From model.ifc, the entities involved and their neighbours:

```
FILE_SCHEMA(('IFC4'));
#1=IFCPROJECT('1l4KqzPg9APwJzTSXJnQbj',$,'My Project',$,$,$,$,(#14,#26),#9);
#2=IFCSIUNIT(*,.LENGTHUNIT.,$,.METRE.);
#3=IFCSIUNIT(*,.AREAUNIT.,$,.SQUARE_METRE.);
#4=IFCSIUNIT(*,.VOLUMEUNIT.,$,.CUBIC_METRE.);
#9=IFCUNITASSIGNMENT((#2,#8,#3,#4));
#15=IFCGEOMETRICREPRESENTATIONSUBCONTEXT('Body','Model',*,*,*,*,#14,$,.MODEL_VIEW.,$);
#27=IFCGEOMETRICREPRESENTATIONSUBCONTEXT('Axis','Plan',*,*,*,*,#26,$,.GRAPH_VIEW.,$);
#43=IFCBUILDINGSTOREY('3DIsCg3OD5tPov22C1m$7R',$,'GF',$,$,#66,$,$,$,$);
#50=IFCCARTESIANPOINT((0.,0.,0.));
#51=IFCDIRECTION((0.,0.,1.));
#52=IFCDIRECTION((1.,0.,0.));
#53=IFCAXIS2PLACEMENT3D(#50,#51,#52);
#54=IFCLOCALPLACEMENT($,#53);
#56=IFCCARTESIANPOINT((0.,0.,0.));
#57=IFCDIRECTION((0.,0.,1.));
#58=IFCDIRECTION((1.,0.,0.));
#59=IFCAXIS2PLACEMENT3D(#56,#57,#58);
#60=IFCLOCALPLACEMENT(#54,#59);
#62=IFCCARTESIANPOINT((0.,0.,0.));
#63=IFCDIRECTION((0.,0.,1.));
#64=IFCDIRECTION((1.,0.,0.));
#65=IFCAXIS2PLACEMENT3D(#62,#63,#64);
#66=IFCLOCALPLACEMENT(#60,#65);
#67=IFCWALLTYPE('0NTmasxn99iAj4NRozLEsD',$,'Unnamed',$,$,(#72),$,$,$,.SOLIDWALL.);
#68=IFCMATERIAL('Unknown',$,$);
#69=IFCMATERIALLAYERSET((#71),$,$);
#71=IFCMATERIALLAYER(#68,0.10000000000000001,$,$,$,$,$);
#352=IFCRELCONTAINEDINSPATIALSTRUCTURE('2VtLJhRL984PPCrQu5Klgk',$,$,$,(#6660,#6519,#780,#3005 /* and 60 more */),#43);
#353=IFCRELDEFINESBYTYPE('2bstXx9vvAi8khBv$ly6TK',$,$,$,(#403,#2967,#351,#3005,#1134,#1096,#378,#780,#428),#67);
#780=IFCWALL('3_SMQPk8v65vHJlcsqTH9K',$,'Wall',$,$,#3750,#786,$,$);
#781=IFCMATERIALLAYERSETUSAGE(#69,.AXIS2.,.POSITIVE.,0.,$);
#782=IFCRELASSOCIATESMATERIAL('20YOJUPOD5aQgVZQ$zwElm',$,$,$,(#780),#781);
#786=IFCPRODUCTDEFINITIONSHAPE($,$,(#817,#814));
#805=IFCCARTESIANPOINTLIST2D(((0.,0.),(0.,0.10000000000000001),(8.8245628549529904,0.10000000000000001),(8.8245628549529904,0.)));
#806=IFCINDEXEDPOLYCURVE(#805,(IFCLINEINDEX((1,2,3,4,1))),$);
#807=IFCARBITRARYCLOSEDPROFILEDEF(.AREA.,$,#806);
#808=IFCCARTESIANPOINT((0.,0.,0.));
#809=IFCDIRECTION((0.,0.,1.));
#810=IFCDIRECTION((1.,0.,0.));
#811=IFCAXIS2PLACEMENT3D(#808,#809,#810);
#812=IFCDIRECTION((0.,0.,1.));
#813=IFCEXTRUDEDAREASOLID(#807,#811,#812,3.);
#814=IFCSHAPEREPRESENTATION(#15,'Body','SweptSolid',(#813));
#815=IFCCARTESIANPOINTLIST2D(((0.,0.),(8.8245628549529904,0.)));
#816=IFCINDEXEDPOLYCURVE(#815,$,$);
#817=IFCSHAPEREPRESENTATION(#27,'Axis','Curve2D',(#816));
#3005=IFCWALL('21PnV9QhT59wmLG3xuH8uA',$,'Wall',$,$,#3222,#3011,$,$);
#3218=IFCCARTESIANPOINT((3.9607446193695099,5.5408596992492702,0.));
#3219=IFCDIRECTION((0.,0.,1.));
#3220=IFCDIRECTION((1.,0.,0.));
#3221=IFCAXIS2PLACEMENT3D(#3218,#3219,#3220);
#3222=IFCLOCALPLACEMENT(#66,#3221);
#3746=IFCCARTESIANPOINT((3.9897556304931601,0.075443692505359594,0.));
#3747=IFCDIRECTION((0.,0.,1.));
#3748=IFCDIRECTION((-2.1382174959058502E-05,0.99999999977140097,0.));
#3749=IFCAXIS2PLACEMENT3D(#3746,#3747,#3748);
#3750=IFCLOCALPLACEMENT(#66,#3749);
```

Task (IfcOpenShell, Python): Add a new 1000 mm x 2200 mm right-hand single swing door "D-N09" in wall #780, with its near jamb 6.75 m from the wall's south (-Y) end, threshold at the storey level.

```python
import numpy as np
import ifcopenshell
import ifcopenshell.api.feature
import ifcopenshell.api.geometry
import ifcopenshell.api.root
import ifcopenshell.api.spatial
import ifcopenshell.geom
import ifcopenshell.util.element
import ifcopenshell.util.placement
import ifcopenshell.util.representation
import ifcopenshell.util.shape
import ifcopenshell.util.unit

model = ifcopenshell.open("model.ifc")
unit_scale = ifcopenshell.util.unit.calculate_unit_scale(model)
settings = ifcopenshell.geom.settings()


def volume(element):
    """Net volume in cubic metres, openings subtracted."""
    shape = ifcopenshell.geom.create_shape(settings, element)
    return ifcopenshell.util.shape.get_volume(shape.geometry)


wall = model.by_id(780)
storey = ifcopenshell.util.element.get_container(wall, ifc_class="IfcBuildingStorey")
context = ifcopenshell.util.representation.get_context(model, "Model", "Body", "MODEL_VIEW")
before = volume(wall)

width, height, from_end, sill = 1, 2.2, 6.75, 0.0  # metres

# The wall runs along its own X axis, and the end named is its -X end.
wall_shape = ifcopenshell.geom.create_shape(settings, wall)
x, y, z = ifcopenshell.util.shape.get_vertices(wall_shape.geometry).T
start = x.min() + from_end
face, thickness = float(y.min()), float(y.max() - y.min())
wall_matrix = ifcopenshell.util.placement.get_local_placement(wall.ObjectPlacement)
level = ifcopenshell.util.placement.get_local_placement(storey.ObjectPlacement)[2, 3]


def in_wall(x, y):
    """Placement at x, y metres in the wall's axes, at sill height."""
    matrix = wall_matrix.copy()
    matrix[:, 3] = wall_matrix @ np.array([x / unit_scale, y / unit_scale, 0.0, 1.0])
    matrix[2, 3] = level + sill / unit_scale
    return matrix


# Opening: a box that overshoots both wall faces by 50 mm.
opening = ifcopenshell.api.root.create_entity(model, ifc_class="IfcOpeningElement", predefined_type="OPENING")
box = ifcopenshell.api.geometry.add_wall_representation(
    model, context=context, length=width, height=height, thickness=thickness + 0.1
)
ifcopenshell.api.geometry.assign_representation(model, product=opening, representation=box)
ifcopenshell.api.geometry.edit_object_placement(model, product=opening, matrix=in_wall(start, face - 0.05), is_si=False)
ifcopenshell.api.feature.add_feature(model, feature=opening, element=wall)

door = ifcopenshell.api.root.create_entity(model, ifc_class="IfcDoor", name="D-N09", predefined_type="DOOR")
door.OverallWidth, door.OverallHeight = width / unit_scale, height / unit_scale
door.OperationType = "SINGLE_SWING_RIGHT"
body = ifcopenshell.api.geometry.add_door_representation(
    model,
    context=context,
    overall_width=door.OverallWidth,
    overall_height=door.OverallHeight,
    operation_type="SINGLE_SWING_RIGHT",
    lining_properties={"LiningDepth": thickness / unit_scale, "ThresholdDepth": thickness / unit_scale},
)
ifcopenshell.api.geometry.assign_representation(model, product=door, representation=body)
ifcopenshell.api.spatial.assign_container(model, products=[door], relating_structure=storey)
ifcopenshell.api.feature.add_filling(model, opening=opening, element=door)

# The lining spans the wall, so the door starts at the wall face.
ifcopenshell.api.geometry.edit_object_placement(model, product=door, matrix=in_wall(start, face), is_si=False)

after = volume(wall)

print(f"wall volume {before:.3f} -> {after:.3f} m3")

model.write("model_rev.ifc")
```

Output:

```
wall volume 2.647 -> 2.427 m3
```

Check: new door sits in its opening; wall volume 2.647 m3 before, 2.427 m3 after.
